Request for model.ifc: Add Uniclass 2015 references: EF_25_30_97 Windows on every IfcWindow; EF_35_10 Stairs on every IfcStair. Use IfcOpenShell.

First a look at what the model holds.

```python
import ifcopenshell

model = ifcopenshell.open("model.ifc")
print(model.schema)
print("classifications:", [c.Name for c in model.by_type("IfcClassification")])
for ifc_class in ("IfcDoor", "IfcRoof", "IfcStair", "IfcWall", "IfcWindow"):
    print(ifc_class, len(model.by_type(ifc_class)))
```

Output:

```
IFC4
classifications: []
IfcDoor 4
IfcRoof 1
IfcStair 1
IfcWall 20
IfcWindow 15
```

```python
import ifcopenshell
import ifcopenshell.api.classification

model = ifcopenshell.open("model.ifc")

system = ifcopenshell.api.classification.add_classification(model, classification="Uniclass 2015")

codes = {
    "IfcWindow": ("EF_25_30_97", "Windows"),
    "IfcStair": ("EF_35_10", "Stairs"),
}
for ifc_class, (code, name) in codes.items():
    products = model.by_type(ifc_class)
    ifcopenshell.api.classification.add_reference(
        model, products=products, classification=system, identification=code, name=name
    )
    print(code, len(products))

model.write("model_updated.ifc")
```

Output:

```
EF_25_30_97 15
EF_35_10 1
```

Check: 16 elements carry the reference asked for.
